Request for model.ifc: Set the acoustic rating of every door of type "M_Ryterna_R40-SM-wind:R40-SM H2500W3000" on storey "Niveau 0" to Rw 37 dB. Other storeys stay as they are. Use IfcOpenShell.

First a look at what the model holds.

```python
import ifcopenshell
import ifcopenshell.util.element

model = ifcopenshell.open("model.ifc")
print(model.schema)
storey = next(s for s in model.by_type("IfcBuildingStorey") if s.Name == "Niveau 0")
doors = [e for e in ifcopenshell.util.element.get_decomposition(storey) if e.is_a("IfcDoor")]
seen = {}
for e in doors:
    element_type = ifcopenshell.util.element.get_type(e)
    key = (element_type.Name if element_type != e and element_type else None, ifcopenshell.util.element.get_pset(e, "Pset_DoorCommon", "AcousticRating"))
    seen[key] = seen.get(key, 0) + 1
for (name, value), count in sorted(seen.items(), key=str):
    print(count, "x", name, "|", value)
```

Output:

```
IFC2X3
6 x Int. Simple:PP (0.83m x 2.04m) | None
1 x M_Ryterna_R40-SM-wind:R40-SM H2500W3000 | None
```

```python
import ifcopenshell
import ifcopenshell.api.pset
import ifcopenshell.util.element

model = ifcopenshell.open("model.ifc")

storey = next(s for s in model.by_type("IfcBuildingStorey") if s.Name == "Niveau 0")
doors = [e for e in ifcopenshell.util.element.get_decomposition(storey) if e.is_a("IfcDoor")]

count = 0
for e in doors:
    element_type = ifcopenshell.util.element.get_type(e)
    if element_type in (None, e) or element_type.Name != "M_Ryterna_R40-SM-wind:R40-SM H2500W3000":
        continue
    # add_pset returns the element's existing set when there is one.
    pset = ifcopenshell.api.pset.add_pset(model, product=e, name="Pset_DoorCommon")
    ifcopenshell.api.pset.edit_pset(model, pset=pset, properties={"AcousticRating": "Rw 37 dB"})
    count += 1

print(count, "doors updated")

model.write("model_rev.ifc")
```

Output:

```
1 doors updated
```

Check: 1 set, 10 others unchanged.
